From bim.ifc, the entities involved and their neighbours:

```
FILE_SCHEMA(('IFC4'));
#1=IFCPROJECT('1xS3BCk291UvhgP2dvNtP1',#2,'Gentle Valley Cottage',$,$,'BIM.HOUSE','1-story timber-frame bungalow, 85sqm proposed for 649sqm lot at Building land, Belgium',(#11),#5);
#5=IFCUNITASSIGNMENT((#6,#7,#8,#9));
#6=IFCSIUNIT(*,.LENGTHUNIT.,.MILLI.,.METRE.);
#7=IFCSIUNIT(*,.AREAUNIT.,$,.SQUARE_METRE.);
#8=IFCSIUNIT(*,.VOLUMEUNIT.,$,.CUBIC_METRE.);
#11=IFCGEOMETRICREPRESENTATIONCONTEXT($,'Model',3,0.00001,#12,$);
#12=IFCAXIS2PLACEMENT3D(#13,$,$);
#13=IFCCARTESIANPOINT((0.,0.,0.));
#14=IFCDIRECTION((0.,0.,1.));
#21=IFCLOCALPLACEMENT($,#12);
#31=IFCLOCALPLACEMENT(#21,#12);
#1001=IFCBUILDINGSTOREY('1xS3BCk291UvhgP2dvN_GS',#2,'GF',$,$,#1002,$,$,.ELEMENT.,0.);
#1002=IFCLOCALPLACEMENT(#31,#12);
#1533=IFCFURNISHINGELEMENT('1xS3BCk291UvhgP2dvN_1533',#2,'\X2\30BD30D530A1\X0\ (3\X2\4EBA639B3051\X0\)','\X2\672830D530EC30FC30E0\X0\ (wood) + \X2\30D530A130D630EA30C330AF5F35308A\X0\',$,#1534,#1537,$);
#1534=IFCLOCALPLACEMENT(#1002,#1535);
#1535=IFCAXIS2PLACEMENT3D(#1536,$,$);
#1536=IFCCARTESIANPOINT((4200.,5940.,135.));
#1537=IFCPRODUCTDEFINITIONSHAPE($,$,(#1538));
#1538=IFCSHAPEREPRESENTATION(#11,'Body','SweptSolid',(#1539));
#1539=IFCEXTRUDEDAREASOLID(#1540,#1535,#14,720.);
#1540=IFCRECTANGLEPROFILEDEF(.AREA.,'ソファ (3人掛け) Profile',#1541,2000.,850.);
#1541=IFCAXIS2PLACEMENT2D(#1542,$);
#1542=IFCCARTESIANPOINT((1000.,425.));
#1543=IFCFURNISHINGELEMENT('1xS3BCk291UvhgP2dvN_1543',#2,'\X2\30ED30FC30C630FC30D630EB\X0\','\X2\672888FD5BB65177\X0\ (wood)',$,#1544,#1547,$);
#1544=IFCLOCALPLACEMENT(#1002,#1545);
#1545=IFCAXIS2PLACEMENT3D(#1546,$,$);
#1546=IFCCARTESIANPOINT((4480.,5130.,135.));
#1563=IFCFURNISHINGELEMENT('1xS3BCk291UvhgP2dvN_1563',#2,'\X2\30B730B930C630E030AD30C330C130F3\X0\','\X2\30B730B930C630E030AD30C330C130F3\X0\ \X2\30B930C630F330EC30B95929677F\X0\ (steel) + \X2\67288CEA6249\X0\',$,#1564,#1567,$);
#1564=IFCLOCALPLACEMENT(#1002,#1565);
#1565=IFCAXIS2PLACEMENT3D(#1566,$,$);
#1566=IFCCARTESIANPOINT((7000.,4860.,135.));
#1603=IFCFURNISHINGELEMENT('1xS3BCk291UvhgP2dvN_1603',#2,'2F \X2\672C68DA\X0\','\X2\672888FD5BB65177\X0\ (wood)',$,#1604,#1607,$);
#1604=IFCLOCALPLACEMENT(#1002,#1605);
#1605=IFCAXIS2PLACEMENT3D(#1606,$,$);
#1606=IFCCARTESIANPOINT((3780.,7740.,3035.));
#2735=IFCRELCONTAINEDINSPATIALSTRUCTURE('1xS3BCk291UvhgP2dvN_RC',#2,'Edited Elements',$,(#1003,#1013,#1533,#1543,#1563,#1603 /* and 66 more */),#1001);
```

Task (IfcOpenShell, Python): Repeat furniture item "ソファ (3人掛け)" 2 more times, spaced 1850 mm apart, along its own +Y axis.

```python
import ifcopenshell
import ifcopenshell.api.geometry
import ifcopenshell.api.root
import ifcopenshell.util.element
import ifcopenshell.util.placement

model = ifcopenshell.open("bim.ifc")


def reuse_history(source, copy):
    """copy_class also copies each property set's owner history, people and application; keep the originals."""
    for rel in copy.IsDefinedBy:
        if rel.is_a("IfcRelDefinesByProperties") and (history := rel.RelatingPropertyDefinition.OwnerHistory):
            rel.RelatingPropertyDefinition.OwnerHistory = source.OwnerHistory
            ifcopenshell.util.element.remove_deep2(model, history)


source = model.by_guid("1xS3BCk291UvhgP2dvN_1533")
base = ifcopenshell.util.placement.get_local_placement(source.ObjectPlacement)
step = base[:3, 1] * 1850.0

for i in range(1, 3):
    copy = ifcopenshell.api.root.copy_class(model, product=source)
    copy.Representation = ifcopenshell.util.element.copy_deep(
        model, source.Representation, exclude=["IfcGeometricRepresentationContext", "IfcRepresentationMap"]
    )
    reuse_history(source, copy)
    matrix = base.copy()
    matrix[:3, 3] += i * step
    print("added at", matrix[:3, 3].round(3) + 0.0)
    ifcopenshell.api.geometry.edit_object_placement(model, product=copy, matrix=matrix, is_si=False)

model.write("bim_v2.ifc")
```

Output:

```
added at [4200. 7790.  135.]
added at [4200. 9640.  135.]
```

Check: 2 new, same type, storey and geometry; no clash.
